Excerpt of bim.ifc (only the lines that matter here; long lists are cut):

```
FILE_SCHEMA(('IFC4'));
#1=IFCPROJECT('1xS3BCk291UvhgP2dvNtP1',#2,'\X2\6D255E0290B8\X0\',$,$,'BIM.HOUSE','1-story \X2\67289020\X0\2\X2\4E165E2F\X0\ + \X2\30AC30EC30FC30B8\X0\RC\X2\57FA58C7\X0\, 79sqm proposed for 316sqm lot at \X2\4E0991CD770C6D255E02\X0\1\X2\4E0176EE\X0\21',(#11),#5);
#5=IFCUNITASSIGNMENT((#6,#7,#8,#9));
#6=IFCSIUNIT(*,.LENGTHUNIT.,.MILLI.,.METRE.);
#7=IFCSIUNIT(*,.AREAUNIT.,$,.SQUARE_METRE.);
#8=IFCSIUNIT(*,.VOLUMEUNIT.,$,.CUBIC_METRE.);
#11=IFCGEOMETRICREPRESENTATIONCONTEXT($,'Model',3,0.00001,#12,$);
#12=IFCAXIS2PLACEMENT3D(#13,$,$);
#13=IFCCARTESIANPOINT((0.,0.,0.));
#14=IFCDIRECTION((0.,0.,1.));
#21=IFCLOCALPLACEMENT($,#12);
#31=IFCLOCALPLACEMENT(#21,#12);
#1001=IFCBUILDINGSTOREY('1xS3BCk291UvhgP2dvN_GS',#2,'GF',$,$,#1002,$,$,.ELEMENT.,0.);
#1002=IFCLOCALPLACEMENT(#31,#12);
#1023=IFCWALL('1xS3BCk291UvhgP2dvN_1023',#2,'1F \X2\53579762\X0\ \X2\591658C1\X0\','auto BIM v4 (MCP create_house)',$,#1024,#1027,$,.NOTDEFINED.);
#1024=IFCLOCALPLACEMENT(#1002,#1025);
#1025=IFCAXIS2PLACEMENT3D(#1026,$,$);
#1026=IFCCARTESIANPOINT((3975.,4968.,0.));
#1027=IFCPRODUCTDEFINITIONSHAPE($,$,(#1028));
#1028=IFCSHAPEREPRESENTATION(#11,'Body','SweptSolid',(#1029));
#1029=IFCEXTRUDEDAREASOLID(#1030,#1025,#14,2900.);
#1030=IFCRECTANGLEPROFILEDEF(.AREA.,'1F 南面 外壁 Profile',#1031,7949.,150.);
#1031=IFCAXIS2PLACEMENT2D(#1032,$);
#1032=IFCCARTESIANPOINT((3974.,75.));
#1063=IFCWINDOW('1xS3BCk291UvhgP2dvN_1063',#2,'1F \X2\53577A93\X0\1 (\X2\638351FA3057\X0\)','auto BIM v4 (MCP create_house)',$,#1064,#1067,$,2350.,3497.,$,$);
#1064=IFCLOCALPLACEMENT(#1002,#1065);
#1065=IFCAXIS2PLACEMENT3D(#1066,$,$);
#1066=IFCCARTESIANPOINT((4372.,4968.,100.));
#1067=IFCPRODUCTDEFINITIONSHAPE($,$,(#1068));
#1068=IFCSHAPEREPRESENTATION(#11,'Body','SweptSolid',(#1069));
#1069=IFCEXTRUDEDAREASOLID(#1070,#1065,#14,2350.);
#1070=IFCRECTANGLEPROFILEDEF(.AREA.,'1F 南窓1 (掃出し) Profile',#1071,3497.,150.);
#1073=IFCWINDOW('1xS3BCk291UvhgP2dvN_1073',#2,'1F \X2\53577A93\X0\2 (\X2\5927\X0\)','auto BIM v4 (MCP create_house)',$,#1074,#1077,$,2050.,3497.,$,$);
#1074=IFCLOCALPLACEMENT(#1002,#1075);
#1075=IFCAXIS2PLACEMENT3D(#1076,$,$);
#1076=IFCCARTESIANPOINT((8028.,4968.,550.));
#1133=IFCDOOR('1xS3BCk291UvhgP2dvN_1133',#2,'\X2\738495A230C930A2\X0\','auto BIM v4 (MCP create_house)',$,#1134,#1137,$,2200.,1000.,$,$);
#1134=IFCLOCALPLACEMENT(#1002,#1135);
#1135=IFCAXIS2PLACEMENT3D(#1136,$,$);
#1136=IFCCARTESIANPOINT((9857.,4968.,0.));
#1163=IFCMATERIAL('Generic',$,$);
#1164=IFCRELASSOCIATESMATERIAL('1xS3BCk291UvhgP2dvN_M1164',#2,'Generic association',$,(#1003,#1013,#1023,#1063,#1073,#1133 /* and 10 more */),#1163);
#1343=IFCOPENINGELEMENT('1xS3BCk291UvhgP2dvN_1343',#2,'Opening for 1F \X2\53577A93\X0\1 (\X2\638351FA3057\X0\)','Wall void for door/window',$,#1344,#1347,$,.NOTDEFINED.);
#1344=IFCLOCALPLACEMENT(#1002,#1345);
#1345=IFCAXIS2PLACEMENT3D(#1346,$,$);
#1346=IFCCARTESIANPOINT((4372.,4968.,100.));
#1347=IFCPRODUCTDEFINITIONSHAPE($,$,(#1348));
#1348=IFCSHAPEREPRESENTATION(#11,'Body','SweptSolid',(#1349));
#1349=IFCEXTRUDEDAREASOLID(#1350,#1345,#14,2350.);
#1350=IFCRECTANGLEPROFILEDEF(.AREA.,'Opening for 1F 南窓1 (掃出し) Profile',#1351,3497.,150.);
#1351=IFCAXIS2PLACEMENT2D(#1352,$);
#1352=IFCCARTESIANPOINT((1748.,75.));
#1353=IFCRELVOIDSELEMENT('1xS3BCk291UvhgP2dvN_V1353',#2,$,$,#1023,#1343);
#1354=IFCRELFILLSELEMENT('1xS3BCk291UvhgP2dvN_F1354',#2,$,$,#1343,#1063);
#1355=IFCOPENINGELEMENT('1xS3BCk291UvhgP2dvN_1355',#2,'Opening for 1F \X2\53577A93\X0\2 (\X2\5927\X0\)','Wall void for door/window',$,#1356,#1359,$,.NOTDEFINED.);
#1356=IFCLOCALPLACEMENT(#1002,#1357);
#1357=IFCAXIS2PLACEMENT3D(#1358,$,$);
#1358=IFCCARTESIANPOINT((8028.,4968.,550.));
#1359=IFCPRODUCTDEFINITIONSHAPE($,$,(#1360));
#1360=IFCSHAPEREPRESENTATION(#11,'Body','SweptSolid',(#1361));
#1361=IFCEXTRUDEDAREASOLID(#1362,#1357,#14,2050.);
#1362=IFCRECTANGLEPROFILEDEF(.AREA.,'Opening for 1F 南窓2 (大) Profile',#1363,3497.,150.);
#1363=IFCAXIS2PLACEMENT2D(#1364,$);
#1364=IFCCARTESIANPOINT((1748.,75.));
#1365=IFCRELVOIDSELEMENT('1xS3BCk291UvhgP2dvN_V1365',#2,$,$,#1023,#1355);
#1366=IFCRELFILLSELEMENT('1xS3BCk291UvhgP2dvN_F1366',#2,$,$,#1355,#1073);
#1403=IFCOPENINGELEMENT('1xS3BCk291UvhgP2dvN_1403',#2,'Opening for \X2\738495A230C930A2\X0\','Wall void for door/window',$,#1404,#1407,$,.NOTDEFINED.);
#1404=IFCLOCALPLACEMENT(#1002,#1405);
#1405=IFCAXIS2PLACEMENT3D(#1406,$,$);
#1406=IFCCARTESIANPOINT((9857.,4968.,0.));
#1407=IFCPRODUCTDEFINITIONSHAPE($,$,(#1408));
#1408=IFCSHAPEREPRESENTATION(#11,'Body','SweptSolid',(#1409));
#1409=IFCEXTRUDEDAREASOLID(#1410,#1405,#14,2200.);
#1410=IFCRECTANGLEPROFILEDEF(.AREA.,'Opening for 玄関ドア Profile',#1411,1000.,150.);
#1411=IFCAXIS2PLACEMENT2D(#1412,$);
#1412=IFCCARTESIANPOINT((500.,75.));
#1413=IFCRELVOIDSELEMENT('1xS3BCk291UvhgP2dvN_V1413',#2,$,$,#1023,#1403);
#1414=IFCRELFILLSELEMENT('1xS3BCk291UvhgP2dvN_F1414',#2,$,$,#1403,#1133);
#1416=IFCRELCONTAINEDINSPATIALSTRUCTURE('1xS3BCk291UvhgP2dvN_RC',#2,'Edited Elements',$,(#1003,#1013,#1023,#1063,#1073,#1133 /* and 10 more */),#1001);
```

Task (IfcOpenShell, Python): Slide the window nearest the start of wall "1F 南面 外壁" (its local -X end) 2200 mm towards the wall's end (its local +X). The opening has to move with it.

```python
import ifcopenshell
import ifcopenshell.api.geometry
import ifcopenshell.util.placement
import ifcopenshell.util.unit

model = ifcopenshell.open("bim.ifc")
unit_scale = ifcopenshell.util.unit.calculate_unit_scale(model)

window = model.by_guid("1xS3BCk291UvhgP2dvN_1063")
opening = window.FillsVoids[0].RelatingOpeningElement
wall = opening.VoidsElements[0].RelatingBuildingElement

wall_matrix = ifcopenshell.util.placement.get_local_placement(wall.ObjectPlacement)
shift = wall_matrix[:3, 0] * 2.2 / unit_scale
before = ifcopenshell.util.placement.get_local_placement(window.ObjectPlacement)[:3, 3].copy()

# The window is not placed relative to its opening, so move both.
for product in (opening, window):
    matrix = ifcopenshell.util.placement.get_local_placement(product.ObjectPlacement)
    matrix[:3, 3] += shift
    ifcopenshell.api.geometry.edit_object_placement(model, product=product, matrix=matrix, is_si=False)

after = ifcopenshell.util.placement.get_local_placement(window.ObjectPlacement)[:3, 3]
print("window moved by", (after - before).round(3) + 0.0)

model.write("bim_updated.ifc")
```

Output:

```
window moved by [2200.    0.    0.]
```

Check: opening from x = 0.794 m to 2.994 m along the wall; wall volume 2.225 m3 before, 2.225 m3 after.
